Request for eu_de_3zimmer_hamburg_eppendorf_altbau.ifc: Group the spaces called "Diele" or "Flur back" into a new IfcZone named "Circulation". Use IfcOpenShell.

First a look at what the model holds.

```python
import ifcopenshell

model = ifcopenshell.open("eu_de_3zimmer_hamburg_eppendorf_altbau.ifc")
print(model.schema)
seen = {}
for space in model.by_type("IfcSpace"):
    seen[space.LongName] = seen.get(space.LongName, 0) + 1
for name, count in sorted(seen.items(), key=str):
    print(count, "x", name)
print("zones:", [z.Name for z in model.by_type("IfcZone")][:20])
```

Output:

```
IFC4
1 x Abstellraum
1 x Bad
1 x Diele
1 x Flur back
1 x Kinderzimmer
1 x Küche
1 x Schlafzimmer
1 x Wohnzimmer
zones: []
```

```python
import ifcopenshell
import ifcopenshell.api.group
import ifcopenshell.api.root

model = ifcopenshell.open("eu_de_3zimmer_hamburg_eppendorf_altbau.ifc")

names = {"Diele", "Flur back"}
spaces = [s for s in model.by_type("IfcSpace") if s.LongName in names]

zone = ifcopenshell.api.root.create_entity(model, ifc_class="IfcZone", name="Circulation")
ifcopenshell.api.group.assign_group(model, products=spaces, group=zone)
print(len(spaces), "spaces in", zone.Name)

model.write("eu_de_3zimmer_hamburg_eppendorf_altbau_v2.ifc")
```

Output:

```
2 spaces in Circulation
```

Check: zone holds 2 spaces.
